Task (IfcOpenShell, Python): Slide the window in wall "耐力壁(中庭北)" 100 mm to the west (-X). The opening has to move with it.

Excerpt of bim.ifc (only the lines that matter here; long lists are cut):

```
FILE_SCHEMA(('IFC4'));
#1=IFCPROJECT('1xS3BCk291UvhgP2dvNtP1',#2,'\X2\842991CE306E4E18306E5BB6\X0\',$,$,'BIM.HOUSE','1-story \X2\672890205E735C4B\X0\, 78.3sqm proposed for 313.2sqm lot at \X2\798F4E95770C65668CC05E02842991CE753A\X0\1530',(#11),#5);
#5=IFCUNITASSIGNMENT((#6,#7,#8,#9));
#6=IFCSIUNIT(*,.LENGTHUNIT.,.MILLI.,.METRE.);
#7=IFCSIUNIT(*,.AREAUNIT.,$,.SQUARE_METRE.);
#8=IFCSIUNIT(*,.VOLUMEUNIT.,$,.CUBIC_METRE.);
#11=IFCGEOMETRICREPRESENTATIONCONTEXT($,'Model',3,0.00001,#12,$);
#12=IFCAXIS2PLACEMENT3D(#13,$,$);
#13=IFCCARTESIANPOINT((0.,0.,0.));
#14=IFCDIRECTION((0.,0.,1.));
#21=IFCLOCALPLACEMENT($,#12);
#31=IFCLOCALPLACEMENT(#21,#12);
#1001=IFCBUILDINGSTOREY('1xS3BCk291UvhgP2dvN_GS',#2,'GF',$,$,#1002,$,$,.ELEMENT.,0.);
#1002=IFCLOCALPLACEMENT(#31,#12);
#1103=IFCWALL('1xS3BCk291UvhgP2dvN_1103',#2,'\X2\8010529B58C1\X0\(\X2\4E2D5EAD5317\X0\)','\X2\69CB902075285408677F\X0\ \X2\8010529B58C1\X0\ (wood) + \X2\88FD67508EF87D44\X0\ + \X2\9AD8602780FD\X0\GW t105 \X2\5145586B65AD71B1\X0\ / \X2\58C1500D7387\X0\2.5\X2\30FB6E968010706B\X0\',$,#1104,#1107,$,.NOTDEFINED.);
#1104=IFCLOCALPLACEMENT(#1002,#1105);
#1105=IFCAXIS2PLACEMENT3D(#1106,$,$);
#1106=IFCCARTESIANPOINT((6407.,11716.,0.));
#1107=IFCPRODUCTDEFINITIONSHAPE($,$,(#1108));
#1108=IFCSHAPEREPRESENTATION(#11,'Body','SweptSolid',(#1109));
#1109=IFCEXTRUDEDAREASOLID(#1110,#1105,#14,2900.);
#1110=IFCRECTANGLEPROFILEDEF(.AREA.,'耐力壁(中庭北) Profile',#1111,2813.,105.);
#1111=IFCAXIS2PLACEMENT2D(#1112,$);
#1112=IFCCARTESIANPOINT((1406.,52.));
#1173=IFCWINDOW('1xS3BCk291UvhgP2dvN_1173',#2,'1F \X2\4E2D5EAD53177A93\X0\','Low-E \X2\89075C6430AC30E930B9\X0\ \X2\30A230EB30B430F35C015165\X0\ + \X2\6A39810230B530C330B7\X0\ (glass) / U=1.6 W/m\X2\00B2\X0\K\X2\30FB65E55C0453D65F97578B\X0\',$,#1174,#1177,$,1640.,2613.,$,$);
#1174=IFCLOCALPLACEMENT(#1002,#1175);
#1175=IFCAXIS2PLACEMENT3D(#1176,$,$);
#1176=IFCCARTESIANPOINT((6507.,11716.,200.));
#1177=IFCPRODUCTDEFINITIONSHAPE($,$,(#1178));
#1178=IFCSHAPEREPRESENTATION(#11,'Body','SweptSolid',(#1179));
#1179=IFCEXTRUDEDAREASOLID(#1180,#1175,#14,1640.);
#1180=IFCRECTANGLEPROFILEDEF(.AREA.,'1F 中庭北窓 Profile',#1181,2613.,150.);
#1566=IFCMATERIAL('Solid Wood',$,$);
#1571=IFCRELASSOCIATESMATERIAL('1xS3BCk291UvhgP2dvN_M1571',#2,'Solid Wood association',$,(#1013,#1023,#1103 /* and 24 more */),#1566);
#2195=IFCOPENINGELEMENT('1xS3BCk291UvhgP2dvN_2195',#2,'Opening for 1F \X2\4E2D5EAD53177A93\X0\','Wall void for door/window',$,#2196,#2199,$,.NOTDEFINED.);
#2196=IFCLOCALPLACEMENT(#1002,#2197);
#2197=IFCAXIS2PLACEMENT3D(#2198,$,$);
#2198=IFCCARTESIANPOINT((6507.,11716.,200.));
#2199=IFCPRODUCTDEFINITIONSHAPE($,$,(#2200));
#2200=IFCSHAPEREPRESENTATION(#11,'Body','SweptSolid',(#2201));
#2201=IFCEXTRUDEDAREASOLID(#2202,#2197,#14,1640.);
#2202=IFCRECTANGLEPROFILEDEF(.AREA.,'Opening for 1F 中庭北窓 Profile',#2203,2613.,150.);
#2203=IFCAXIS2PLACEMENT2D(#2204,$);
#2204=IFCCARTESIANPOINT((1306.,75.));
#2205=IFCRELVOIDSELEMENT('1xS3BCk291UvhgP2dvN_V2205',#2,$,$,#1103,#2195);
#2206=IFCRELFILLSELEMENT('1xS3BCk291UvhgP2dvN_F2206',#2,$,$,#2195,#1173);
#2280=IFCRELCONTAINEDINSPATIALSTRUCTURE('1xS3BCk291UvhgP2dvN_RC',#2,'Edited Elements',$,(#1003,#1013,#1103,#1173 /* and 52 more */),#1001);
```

```python
import ifcopenshell
import ifcopenshell.api.geometry
import ifcopenshell.util.placement

model = ifcopenshell.open("bim.ifc")

window = model.by_guid("1xS3BCk291UvhgP2dvN_1173")
opening = window.FillsVoids[0].RelatingOpeningElement
wall = opening.VoidsElements[0].RelatingBuildingElement

wall_matrix = ifcopenshell.util.placement.get_local_placement(wall.ObjectPlacement)
shift = wall_matrix[:3, 0] * -100.0
before = ifcopenshell.util.placement.get_local_placement(window.ObjectPlacement)[:3, 3].copy()

# The window is not placed relative to its opening, so move both.
for product in (opening, window):
    matrix = ifcopenshell.util.placement.get_local_placement(product.ObjectPlacement)
    matrix[:3, 3] += shift
    ifcopenshell.api.geometry.edit_object_placement(model, product=product, matrix=matrix, is_si=False)

after = ifcopenshell.util.placement.get_local_placement(window.ObjectPlacement)[:3, 3]
print("window moved by", (after - before).round(3) + 0.0)

model.write("bim_rev.ifc")
```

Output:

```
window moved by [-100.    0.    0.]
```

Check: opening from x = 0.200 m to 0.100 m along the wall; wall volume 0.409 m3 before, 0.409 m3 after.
